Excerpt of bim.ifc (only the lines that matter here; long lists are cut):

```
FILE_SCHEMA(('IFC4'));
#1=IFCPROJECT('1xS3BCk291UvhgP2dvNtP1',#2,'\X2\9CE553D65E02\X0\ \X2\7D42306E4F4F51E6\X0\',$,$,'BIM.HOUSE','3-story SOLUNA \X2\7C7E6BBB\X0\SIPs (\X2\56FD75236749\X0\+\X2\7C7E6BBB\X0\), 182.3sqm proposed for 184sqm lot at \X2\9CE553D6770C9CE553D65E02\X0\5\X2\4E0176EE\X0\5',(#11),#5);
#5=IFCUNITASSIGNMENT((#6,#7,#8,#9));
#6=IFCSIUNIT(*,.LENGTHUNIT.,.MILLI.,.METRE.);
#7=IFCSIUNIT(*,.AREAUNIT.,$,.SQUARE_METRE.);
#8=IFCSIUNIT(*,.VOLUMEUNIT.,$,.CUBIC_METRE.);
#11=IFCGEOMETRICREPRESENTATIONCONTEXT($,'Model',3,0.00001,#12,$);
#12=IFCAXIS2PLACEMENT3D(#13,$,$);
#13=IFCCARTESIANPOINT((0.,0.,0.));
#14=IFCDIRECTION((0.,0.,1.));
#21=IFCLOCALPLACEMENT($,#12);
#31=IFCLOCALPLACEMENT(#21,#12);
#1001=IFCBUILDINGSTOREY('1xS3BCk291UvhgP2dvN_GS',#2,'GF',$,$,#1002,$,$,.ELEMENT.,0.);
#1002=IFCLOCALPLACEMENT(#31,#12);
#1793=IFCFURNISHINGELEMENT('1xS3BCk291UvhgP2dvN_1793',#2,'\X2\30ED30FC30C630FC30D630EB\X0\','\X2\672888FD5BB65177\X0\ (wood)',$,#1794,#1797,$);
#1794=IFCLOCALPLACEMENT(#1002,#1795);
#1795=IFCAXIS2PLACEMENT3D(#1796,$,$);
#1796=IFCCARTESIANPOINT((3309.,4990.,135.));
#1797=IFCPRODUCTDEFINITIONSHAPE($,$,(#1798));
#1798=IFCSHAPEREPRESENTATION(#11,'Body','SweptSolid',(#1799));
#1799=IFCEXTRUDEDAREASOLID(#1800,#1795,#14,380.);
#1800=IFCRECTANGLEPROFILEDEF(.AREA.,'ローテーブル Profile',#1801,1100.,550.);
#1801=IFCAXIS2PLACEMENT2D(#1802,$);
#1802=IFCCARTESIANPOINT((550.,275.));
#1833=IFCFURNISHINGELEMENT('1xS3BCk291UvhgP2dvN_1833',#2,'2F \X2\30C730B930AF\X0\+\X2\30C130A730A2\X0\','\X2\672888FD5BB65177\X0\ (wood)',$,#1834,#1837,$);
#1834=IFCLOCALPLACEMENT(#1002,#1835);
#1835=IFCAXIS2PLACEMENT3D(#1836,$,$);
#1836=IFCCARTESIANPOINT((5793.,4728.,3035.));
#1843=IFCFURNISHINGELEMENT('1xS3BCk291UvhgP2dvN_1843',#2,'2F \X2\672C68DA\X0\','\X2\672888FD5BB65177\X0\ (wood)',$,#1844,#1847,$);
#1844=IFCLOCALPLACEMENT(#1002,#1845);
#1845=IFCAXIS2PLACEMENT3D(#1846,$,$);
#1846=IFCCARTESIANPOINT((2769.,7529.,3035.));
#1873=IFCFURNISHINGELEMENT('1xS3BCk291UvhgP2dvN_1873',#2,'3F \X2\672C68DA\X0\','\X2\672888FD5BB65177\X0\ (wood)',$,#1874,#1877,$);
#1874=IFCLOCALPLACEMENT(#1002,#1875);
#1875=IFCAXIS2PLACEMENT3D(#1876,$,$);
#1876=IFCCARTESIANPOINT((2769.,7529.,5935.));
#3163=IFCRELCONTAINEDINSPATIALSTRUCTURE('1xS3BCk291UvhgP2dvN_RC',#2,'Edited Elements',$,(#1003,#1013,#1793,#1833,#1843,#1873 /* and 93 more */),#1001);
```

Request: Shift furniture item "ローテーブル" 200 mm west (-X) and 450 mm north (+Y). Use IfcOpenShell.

```python
import ifcopenshell
import ifcopenshell.api.geometry
import ifcopenshell.util.placement

model = ifcopenshell.open("bim.ifc")

item = model.by_guid("1xS3BCk291UvhgP2dvN_1793")
matrix = ifcopenshell.util.placement.get_local_placement(item.ObjectPlacement)
matrix[0, 3] -= 200.0
matrix[1, 3] += 450.0
ifcopenshell.api.geometry.edit_object_placement(model, product=item, matrix=matrix, is_si=False)

print(ifcopenshell.util.placement.get_local_placement(item.ObjectPlacement).round(3) + 0.0)

model.write("bim-out.ifc")
```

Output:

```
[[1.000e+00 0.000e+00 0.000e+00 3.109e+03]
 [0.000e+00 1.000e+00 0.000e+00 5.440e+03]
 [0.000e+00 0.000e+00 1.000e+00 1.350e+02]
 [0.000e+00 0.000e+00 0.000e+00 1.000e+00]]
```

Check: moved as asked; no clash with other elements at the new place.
